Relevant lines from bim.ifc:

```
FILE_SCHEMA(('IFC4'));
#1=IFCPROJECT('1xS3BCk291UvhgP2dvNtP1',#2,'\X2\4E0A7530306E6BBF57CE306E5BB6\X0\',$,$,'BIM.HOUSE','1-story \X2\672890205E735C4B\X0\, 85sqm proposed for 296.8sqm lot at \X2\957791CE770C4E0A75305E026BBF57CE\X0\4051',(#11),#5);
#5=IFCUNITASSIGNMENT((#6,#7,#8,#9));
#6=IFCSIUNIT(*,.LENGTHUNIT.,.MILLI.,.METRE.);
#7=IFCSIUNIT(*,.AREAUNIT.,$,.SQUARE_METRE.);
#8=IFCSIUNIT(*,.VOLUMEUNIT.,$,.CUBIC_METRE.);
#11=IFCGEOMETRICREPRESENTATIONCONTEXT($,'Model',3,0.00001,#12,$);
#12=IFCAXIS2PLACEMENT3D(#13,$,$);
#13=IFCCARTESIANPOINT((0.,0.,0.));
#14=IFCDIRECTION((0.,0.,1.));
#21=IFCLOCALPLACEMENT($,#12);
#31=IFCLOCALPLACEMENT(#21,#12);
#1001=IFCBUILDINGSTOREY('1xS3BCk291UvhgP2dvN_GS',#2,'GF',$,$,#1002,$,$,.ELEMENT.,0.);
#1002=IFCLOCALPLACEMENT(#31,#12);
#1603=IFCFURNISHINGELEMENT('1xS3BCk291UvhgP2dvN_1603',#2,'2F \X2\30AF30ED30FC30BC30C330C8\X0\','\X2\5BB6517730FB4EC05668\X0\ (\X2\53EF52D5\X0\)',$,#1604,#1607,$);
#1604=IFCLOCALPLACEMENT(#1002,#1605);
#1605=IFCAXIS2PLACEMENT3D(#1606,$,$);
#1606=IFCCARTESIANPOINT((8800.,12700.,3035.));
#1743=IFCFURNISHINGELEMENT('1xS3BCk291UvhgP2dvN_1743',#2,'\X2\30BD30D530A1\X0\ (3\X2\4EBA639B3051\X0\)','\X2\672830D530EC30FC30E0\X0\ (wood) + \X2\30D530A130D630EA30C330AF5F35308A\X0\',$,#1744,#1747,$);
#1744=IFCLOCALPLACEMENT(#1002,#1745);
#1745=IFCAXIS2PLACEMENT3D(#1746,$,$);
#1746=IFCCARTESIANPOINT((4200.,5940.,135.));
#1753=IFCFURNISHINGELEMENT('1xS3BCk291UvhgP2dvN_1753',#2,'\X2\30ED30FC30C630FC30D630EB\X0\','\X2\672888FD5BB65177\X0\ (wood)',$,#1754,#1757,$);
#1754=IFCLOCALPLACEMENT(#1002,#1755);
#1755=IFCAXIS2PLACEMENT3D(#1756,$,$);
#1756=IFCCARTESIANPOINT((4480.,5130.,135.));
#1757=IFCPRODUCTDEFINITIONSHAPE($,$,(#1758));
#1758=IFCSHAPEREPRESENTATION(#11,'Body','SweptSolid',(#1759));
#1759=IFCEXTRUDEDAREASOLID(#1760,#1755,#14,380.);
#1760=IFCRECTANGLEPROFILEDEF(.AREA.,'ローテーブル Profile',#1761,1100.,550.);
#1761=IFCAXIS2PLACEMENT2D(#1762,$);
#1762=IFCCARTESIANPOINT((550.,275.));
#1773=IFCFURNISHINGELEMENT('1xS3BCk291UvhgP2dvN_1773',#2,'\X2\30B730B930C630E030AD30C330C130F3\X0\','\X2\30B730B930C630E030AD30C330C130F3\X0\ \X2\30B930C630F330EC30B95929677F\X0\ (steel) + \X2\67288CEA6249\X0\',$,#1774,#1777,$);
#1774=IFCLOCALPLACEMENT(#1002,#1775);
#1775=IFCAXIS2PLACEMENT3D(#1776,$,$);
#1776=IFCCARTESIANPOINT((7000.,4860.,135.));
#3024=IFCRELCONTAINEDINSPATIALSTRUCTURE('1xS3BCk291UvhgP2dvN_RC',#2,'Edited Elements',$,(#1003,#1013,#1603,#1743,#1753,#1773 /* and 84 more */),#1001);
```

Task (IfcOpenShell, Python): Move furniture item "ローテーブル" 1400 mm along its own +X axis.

```python
import ifcopenshell
import ifcopenshell.api.geometry
import ifcopenshell.util.placement

model = ifcopenshell.open("bim.ifc")

item = model.by_guid("1xS3BCk291UvhgP2dvN_1753")
matrix = ifcopenshell.util.placement.get_local_placement(item.ObjectPlacement)
matrix[:3, 3] += matrix[:3, 0] * 1400.0
ifcopenshell.api.geometry.edit_object_placement(model, product=item, matrix=matrix, is_si=False)

print(ifcopenshell.util.placement.get_local_placement(item.ObjectPlacement).round(3) + 0.0)

model.write("bim_updated.ifc")
```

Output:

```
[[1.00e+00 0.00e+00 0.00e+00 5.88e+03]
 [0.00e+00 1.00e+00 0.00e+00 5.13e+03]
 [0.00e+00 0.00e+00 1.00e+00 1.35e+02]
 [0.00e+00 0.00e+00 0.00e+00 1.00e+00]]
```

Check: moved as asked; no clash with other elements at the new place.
